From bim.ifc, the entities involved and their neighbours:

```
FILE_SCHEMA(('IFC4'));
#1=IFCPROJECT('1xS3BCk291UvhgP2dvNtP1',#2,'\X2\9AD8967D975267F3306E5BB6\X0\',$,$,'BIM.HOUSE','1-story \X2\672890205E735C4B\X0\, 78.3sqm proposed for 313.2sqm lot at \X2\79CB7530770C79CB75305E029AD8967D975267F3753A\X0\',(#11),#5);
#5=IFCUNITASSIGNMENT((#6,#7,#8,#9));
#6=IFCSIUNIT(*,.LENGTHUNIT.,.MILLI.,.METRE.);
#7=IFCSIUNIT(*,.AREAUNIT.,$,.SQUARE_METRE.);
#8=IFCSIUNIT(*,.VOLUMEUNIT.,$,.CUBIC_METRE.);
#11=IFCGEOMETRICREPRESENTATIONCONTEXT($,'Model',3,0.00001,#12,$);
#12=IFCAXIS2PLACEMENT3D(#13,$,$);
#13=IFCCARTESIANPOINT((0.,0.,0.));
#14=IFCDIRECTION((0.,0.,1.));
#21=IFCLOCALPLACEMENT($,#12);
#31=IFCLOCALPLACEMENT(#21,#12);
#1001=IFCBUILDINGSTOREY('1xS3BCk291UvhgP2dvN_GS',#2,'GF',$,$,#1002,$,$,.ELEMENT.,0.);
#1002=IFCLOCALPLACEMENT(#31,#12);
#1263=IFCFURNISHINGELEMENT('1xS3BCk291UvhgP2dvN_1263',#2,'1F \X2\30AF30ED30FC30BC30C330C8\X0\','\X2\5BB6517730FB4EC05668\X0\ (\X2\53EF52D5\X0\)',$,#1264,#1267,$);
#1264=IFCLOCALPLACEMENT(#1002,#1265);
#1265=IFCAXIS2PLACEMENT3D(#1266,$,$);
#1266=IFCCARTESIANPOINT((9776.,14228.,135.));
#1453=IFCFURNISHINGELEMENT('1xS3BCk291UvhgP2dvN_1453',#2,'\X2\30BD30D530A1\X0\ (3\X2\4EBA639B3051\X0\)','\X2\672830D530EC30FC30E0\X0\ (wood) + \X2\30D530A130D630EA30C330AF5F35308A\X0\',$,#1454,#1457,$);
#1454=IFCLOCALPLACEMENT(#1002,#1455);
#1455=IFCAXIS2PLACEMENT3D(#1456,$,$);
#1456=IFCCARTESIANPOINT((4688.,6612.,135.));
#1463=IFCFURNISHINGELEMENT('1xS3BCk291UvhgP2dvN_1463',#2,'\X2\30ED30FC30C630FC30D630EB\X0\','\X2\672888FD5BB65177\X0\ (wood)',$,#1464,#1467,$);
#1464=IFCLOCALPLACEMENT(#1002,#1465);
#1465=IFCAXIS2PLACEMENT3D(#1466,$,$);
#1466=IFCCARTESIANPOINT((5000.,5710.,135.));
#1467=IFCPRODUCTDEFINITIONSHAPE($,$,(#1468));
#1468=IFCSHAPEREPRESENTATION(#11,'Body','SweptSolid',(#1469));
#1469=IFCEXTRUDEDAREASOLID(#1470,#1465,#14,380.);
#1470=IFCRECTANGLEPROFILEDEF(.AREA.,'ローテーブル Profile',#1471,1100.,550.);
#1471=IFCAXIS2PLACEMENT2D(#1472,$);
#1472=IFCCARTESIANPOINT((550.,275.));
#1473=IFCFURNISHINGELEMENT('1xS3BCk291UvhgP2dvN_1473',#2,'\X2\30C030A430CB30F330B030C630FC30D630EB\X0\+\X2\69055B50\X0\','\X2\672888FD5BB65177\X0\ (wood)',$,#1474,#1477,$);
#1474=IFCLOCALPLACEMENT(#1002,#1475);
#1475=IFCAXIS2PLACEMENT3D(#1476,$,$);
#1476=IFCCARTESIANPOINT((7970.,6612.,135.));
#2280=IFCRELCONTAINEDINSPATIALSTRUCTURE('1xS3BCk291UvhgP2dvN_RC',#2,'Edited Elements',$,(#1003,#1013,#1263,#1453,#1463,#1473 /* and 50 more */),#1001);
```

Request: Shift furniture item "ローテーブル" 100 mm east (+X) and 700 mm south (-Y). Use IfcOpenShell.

```python
import ifcopenshell
import ifcopenshell.api.geometry
import ifcopenshell.util.placement

model = ifcopenshell.open("bim.ifc")

item = model.by_guid("1xS3BCk291UvhgP2dvN_1463")
matrix = ifcopenshell.util.placement.get_local_placement(item.ObjectPlacement)
matrix[0, 3] += 100.0
matrix[1, 3] -= 700.0
ifcopenshell.api.geometry.edit_object_placement(model, product=item, matrix=matrix, is_si=False)

print(ifcopenshell.util.placement.get_local_placement(item.ObjectPlacement).round(3) + 0.0)

model.write("bim_rev.ifc")
```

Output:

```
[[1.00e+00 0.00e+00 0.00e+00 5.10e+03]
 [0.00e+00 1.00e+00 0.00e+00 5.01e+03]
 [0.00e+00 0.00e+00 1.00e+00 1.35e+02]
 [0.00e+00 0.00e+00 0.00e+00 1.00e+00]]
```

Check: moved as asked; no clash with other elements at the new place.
